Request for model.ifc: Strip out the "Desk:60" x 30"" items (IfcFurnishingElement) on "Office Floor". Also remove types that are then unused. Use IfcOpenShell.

First a look at what the model holds.

```python
import ifcopenshell
import ifcopenshell.util.element

model = ifcopenshell.open("model.ifc")
print(model.schema)
storey = next(s for s in model.by_type("IfcBuildingStorey") if s.Name == "Office Floor")
furniture = [e for e in ifcopenshell.util.element.get_decomposition(storey) if e.is_a("IfcFurnishingElement")]
seen = {}
for e in furniture:
    element_type = ifcopenshell.util.element.get_type(e)
    name = element_type.Name if element_type not in (None, e) else None
    seen[name] = seen.get(name, 0) + 1
for name, count in sorted(seen.items(), key=str):
    print(count, "x", name)
```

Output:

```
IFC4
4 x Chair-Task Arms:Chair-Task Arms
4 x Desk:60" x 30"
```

```python
import ifcopenshell
import ifcopenshell.api.root
import ifcopenshell.util.element

model = ifcopenshell.open("model.ifc")

storey = next(s for s in model.by_type("IfcBuildingStorey") if s.Name == "Office Floor")
furniture = [e for e in ifcopenshell.util.element.get_decomposition(storey) if e.is_a("IfcFurnishingElement")]
targets = [e for e in furniture if (t := ifcopenshell.util.element.get_type(e)) not in (None, e) and t.Name == 'Desk:60" x 30"']
types = {ifcopenshell.util.element.get_type(e) for e in targets} - {None, *targets}

for e in targets:
    ifcopenshell.api.root.remove_product(model, product=e)
print(len(targets), "removed")

unused = [t for t in types if not ifcopenshell.util.element.get_types(t)]
for t in unused:
    ifcopenshell.api.root.remove_product(model, product=t)
print(len(unused), "unused types removed")

model.write("model-out.ifc")
```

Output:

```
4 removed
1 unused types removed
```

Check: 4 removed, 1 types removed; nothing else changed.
